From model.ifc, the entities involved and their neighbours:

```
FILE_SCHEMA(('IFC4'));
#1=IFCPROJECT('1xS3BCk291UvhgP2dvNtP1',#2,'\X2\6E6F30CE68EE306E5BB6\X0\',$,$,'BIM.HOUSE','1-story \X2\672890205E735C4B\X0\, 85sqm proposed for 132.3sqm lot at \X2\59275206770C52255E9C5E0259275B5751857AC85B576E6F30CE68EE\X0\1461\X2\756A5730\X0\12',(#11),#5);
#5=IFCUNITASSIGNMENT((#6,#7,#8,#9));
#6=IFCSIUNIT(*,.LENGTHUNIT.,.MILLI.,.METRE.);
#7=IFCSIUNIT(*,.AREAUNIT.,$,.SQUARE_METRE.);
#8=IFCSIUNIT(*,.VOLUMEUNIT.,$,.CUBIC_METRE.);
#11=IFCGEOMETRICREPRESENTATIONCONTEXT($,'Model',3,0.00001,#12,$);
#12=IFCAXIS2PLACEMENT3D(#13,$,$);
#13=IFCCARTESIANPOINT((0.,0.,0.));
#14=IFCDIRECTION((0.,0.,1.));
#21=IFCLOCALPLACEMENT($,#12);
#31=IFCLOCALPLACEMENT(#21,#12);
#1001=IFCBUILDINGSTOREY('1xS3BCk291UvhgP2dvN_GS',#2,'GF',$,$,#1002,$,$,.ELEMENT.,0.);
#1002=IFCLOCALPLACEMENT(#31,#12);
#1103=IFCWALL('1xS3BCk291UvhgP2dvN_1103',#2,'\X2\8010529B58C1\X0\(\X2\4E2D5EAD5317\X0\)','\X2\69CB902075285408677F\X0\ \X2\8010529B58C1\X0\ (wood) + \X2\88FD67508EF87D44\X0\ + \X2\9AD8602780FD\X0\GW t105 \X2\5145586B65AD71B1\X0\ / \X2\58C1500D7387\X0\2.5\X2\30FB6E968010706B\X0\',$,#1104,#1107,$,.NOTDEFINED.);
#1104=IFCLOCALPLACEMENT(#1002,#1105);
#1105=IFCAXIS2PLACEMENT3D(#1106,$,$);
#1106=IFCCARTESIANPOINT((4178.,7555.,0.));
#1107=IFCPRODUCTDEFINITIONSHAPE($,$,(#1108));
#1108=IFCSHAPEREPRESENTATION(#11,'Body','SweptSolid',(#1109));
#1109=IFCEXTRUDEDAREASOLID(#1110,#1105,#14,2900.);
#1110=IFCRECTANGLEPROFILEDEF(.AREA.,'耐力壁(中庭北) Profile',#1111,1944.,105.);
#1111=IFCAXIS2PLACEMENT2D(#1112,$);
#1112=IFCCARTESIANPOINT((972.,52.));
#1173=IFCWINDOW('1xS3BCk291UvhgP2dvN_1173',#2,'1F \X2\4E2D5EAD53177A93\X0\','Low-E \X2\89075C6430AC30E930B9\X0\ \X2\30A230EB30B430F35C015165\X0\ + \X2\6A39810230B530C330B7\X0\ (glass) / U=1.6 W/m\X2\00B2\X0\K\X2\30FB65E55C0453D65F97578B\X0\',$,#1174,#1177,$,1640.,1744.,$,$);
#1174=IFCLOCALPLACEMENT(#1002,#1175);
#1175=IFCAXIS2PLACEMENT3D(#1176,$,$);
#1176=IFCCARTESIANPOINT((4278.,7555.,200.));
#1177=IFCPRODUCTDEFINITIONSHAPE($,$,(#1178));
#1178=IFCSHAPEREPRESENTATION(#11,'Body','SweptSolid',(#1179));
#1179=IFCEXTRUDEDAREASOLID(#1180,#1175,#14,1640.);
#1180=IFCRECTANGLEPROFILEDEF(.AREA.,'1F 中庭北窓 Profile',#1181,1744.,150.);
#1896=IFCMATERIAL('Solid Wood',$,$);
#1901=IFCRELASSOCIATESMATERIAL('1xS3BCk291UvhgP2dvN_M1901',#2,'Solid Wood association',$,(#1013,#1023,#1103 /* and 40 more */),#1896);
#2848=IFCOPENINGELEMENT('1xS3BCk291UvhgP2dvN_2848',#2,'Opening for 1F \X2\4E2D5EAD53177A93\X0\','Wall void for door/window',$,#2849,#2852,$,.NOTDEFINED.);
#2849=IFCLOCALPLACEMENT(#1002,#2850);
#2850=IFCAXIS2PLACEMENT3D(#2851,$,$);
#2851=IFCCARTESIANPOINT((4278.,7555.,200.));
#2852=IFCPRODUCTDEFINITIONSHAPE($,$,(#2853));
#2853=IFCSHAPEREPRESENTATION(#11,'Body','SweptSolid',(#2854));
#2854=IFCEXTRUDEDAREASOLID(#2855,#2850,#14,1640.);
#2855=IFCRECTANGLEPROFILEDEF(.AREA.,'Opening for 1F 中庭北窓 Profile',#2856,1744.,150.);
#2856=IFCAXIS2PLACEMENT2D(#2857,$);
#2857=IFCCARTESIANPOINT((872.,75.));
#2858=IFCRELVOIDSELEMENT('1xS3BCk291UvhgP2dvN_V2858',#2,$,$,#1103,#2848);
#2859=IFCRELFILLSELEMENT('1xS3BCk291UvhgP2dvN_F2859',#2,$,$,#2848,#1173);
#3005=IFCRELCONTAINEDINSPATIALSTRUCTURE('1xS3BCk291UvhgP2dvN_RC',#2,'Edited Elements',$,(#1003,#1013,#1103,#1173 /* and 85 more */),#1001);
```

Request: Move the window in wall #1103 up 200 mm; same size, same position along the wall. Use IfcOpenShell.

```python
import numpy as np
import ifcopenshell
import ifcopenshell.api.geometry
import ifcopenshell.util.placement
import ifcopenshell.util.unit

model = ifcopenshell.open("model.ifc")
unit_scale = ifcopenshell.util.unit.calculate_unit_scale(model)

window = model.by_guid("1xS3BCk291UvhgP2dvN_1173")
opening = window.FillsVoids[0].RelatingOpeningElement
dz = 0.2 / unit_scale

shift = np.array([0.0, 0.0, dz])
# The window is not placed relative to its opening, so move both.
for product in (opening, window):
    matrix = ifcopenshell.util.placement.get_local_placement(product.ObjectPlacement)
    matrix[:3, 3] += shift
    ifcopenshell.api.geometry.edit_object_placement(model, product=product, matrix=matrix, is_si=False)

print(f"moved by {dz * unit_scale:+.3f} m")

model.write("model_v2.ifc")
```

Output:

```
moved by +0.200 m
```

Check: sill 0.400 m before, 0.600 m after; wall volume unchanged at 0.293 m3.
